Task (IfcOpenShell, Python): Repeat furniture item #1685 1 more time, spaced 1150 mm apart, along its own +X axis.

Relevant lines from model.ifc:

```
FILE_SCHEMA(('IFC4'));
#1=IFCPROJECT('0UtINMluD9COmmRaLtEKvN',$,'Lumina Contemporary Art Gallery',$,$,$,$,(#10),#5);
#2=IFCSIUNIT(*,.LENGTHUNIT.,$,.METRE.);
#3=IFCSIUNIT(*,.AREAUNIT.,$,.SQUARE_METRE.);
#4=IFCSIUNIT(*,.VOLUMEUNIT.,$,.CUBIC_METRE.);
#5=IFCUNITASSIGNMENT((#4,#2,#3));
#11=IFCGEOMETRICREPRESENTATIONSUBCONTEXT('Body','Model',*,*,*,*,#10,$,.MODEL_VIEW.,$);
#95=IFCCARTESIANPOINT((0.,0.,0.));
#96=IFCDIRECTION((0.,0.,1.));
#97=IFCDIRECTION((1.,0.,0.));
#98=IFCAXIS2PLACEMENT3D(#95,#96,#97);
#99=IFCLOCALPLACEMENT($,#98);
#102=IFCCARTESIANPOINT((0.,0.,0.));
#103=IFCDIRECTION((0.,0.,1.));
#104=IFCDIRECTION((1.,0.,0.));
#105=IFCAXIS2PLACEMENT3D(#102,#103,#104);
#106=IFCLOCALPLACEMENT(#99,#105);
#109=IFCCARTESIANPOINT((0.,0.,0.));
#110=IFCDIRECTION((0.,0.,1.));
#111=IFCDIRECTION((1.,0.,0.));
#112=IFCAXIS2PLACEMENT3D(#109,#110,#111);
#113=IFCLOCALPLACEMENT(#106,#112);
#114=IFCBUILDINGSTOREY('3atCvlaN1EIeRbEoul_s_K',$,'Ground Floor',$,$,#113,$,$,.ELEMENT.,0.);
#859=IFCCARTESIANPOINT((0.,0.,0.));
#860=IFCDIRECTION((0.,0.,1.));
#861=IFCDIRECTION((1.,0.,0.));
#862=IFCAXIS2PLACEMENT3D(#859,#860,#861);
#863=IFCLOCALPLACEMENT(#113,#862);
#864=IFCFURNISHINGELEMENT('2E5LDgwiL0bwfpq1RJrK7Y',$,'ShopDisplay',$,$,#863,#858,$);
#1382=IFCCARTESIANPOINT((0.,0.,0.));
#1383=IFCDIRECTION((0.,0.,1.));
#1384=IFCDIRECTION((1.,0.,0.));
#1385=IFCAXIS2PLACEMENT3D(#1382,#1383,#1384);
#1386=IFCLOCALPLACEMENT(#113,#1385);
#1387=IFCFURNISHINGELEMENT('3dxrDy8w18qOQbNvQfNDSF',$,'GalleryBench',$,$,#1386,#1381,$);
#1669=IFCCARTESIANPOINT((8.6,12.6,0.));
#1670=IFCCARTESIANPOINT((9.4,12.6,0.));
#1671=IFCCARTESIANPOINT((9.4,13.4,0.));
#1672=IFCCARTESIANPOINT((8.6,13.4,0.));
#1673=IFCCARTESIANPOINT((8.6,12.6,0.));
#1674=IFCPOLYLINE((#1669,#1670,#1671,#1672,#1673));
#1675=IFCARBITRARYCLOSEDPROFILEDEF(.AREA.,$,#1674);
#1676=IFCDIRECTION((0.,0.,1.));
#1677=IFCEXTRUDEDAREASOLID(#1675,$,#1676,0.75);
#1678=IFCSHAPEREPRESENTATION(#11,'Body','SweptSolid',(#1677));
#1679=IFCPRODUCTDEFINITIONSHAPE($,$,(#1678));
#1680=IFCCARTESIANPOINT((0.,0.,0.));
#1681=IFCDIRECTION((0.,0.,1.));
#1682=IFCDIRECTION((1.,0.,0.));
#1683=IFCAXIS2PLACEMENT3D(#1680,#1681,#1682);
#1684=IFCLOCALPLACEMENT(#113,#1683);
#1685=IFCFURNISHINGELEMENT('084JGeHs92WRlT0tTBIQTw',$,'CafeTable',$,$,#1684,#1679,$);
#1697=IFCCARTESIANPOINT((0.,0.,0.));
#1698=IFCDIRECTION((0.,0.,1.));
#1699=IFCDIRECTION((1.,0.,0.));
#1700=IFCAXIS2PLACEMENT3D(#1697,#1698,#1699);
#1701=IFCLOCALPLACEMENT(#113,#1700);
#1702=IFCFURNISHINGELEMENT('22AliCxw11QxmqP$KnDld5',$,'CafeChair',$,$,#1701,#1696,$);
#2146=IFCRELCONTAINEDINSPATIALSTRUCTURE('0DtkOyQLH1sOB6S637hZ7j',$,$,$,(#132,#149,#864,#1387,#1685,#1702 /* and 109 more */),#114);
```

```python
import ifcopenshell
import ifcopenshell.api.geometry
import ifcopenshell.api.root
import ifcopenshell.util.element
import ifcopenshell.util.placement

model = ifcopenshell.open("model.ifc")

source = model.by_guid("084JGeHs92WRlT0tTBIQTw")
base = ifcopenshell.util.placement.get_local_placement(source.ObjectPlacement)
step = base[:3, 0] * 1.15

for i in range(1, 2):
    copy = ifcopenshell.api.root.copy_class(model, product=source)
    copy.Representation = ifcopenshell.util.element.copy_deep(
        model, source.Representation, exclude=["IfcGeometricRepresentationContext", "IfcRepresentationMap"]
    )
    matrix = base.copy()
    matrix[:3, 3] += i * step
    print("added at", matrix[:3, 3].round(3) + 0.0)
    ifcopenshell.api.geometry.edit_object_placement(model, product=copy, matrix=matrix, is_si=False)

model.write("model_v2.ifc")
```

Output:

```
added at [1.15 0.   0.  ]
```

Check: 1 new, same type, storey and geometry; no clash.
